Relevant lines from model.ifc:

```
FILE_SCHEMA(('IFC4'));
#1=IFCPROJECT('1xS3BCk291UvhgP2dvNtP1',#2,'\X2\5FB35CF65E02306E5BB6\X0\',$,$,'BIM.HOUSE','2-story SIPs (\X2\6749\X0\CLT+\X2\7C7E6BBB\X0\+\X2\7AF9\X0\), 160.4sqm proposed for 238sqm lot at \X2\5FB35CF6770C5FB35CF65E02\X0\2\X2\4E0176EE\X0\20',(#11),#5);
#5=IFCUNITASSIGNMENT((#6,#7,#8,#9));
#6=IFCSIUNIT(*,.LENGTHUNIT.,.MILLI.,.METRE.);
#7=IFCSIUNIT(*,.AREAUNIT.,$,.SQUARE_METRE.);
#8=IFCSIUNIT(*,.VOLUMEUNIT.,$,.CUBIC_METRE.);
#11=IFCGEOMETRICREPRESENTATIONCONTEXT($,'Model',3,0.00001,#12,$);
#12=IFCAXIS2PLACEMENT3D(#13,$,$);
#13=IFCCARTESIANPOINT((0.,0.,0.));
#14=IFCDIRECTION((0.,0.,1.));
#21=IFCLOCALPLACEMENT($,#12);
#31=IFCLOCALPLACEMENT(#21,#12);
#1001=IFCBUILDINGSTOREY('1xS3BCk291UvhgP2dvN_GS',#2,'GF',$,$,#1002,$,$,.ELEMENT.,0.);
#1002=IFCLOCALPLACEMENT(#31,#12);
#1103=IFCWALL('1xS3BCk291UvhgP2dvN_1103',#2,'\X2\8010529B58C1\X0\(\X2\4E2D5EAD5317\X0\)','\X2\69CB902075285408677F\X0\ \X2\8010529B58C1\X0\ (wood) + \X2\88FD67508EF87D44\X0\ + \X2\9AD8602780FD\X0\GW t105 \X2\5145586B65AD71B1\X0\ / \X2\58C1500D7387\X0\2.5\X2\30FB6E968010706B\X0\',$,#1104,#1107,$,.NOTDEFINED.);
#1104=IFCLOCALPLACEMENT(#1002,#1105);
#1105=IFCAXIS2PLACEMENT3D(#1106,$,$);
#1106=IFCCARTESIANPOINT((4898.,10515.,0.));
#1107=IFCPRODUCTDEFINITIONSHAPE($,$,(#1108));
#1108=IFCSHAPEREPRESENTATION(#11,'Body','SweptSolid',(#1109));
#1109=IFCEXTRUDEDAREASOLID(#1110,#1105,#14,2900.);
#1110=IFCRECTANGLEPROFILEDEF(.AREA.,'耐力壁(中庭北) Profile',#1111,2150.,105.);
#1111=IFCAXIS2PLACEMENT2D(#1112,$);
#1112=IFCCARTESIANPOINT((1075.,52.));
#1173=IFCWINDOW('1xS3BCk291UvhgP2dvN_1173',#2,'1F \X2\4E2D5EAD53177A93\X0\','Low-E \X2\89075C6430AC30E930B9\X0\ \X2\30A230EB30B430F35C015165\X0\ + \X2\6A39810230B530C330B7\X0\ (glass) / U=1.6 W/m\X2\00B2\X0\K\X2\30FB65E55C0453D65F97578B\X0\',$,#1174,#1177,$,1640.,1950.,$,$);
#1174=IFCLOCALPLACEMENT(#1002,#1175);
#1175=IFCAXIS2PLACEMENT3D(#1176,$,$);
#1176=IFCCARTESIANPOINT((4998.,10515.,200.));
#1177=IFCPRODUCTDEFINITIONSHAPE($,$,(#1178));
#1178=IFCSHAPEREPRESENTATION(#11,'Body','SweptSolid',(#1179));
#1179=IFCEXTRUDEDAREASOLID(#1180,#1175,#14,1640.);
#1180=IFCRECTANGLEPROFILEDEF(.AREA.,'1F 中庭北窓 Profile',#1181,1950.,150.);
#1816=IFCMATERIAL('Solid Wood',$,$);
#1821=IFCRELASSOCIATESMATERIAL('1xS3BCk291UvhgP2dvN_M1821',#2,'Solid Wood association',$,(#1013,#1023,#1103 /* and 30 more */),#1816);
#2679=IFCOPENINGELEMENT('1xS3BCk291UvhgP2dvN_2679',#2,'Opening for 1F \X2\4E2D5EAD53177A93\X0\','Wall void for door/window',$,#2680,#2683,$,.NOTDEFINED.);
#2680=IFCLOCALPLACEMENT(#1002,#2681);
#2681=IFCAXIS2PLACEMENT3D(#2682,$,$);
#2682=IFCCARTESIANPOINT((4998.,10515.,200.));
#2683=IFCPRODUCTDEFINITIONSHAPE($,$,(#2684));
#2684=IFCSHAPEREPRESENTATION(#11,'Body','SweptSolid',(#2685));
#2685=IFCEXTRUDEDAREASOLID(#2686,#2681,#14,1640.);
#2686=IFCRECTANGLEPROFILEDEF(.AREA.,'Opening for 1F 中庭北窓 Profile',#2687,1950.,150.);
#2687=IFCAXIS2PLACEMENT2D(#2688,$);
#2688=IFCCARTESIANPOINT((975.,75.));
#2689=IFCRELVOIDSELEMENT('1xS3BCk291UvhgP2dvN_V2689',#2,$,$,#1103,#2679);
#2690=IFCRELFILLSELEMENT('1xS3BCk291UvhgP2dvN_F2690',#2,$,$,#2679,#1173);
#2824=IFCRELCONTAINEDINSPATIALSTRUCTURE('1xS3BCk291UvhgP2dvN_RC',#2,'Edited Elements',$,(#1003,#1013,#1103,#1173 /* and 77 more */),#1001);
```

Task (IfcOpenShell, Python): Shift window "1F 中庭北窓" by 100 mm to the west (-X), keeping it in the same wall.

```python
import ifcopenshell
import ifcopenshell.api.geometry
import ifcopenshell.util.placement

model = ifcopenshell.open("model.ifc")

window = model.by_id(1173)
opening = window.FillsVoids[0].RelatingOpeningElement
wall = opening.VoidsElements[0].RelatingBuildingElement

wall_matrix = ifcopenshell.util.placement.get_local_placement(wall.ObjectPlacement)
shift = wall_matrix[:3, 0] * -100.0
before = ifcopenshell.util.placement.get_local_placement(window.ObjectPlacement)[:3, 3].copy()

# The window is not placed relative to its opening, so move both.
for product in (opening, window):
    matrix = ifcopenshell.util.placement.get_local_placement(product.ObjectPlacement)
    matrix[:3, 3] += shift
    ifcopenshell.api.geometry.edit_object_placement(model, product=product, matrix=matrix, is_si=False)

after = ifcopenshell.util.placement.get_local_placement(window.ObjectPlacement)[:3, 3]
print("window moved by", (after - before).round(3) + 0.0)

model.write("model-out.ifc")
```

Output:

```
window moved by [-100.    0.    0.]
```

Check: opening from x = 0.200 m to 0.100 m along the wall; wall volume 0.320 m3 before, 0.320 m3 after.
